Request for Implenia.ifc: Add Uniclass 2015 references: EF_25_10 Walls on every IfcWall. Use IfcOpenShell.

First a look at what the model holds.

```python
import ifcopenshell

model = ifcopenshell.open("Implenia.ifc")
print(model.schema)
print("classifications:", [c.Name for c in model.by_type("IfcClassification")])
for ifc_class in ("IfcDoor", "IfcRoof", "IfcStair", "IfcWall", "IfcWindow"):
    print(ifc_class, len(model.by_type(ifc_class)))
```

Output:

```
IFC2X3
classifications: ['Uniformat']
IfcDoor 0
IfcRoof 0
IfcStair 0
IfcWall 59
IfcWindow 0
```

```python
import ifcopenshell
import ifcopenshell.api.classification

model = ifcopenshell.open("Implenia.ifc")

# IFC2X3 requires Source and Edition and has no link from the project to the system.
system = model.create_entity("IfcClassification", Source="NBS", Edition="2015", Name="Uniclass 2015")

codes = {
    "IfcWall": ("EF_25_10", "Walls"),
}
for ifc_class, (code, name) in codes.items():
    products = model.by_type(ifc_class)
    ifcopenshell.api.classification.add_reference(
        model, products=products, classification=system, identification=code, name=name
    )
    print(code, len(products))

model.write("Implenia_updated.ifc")
```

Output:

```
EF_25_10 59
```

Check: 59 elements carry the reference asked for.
